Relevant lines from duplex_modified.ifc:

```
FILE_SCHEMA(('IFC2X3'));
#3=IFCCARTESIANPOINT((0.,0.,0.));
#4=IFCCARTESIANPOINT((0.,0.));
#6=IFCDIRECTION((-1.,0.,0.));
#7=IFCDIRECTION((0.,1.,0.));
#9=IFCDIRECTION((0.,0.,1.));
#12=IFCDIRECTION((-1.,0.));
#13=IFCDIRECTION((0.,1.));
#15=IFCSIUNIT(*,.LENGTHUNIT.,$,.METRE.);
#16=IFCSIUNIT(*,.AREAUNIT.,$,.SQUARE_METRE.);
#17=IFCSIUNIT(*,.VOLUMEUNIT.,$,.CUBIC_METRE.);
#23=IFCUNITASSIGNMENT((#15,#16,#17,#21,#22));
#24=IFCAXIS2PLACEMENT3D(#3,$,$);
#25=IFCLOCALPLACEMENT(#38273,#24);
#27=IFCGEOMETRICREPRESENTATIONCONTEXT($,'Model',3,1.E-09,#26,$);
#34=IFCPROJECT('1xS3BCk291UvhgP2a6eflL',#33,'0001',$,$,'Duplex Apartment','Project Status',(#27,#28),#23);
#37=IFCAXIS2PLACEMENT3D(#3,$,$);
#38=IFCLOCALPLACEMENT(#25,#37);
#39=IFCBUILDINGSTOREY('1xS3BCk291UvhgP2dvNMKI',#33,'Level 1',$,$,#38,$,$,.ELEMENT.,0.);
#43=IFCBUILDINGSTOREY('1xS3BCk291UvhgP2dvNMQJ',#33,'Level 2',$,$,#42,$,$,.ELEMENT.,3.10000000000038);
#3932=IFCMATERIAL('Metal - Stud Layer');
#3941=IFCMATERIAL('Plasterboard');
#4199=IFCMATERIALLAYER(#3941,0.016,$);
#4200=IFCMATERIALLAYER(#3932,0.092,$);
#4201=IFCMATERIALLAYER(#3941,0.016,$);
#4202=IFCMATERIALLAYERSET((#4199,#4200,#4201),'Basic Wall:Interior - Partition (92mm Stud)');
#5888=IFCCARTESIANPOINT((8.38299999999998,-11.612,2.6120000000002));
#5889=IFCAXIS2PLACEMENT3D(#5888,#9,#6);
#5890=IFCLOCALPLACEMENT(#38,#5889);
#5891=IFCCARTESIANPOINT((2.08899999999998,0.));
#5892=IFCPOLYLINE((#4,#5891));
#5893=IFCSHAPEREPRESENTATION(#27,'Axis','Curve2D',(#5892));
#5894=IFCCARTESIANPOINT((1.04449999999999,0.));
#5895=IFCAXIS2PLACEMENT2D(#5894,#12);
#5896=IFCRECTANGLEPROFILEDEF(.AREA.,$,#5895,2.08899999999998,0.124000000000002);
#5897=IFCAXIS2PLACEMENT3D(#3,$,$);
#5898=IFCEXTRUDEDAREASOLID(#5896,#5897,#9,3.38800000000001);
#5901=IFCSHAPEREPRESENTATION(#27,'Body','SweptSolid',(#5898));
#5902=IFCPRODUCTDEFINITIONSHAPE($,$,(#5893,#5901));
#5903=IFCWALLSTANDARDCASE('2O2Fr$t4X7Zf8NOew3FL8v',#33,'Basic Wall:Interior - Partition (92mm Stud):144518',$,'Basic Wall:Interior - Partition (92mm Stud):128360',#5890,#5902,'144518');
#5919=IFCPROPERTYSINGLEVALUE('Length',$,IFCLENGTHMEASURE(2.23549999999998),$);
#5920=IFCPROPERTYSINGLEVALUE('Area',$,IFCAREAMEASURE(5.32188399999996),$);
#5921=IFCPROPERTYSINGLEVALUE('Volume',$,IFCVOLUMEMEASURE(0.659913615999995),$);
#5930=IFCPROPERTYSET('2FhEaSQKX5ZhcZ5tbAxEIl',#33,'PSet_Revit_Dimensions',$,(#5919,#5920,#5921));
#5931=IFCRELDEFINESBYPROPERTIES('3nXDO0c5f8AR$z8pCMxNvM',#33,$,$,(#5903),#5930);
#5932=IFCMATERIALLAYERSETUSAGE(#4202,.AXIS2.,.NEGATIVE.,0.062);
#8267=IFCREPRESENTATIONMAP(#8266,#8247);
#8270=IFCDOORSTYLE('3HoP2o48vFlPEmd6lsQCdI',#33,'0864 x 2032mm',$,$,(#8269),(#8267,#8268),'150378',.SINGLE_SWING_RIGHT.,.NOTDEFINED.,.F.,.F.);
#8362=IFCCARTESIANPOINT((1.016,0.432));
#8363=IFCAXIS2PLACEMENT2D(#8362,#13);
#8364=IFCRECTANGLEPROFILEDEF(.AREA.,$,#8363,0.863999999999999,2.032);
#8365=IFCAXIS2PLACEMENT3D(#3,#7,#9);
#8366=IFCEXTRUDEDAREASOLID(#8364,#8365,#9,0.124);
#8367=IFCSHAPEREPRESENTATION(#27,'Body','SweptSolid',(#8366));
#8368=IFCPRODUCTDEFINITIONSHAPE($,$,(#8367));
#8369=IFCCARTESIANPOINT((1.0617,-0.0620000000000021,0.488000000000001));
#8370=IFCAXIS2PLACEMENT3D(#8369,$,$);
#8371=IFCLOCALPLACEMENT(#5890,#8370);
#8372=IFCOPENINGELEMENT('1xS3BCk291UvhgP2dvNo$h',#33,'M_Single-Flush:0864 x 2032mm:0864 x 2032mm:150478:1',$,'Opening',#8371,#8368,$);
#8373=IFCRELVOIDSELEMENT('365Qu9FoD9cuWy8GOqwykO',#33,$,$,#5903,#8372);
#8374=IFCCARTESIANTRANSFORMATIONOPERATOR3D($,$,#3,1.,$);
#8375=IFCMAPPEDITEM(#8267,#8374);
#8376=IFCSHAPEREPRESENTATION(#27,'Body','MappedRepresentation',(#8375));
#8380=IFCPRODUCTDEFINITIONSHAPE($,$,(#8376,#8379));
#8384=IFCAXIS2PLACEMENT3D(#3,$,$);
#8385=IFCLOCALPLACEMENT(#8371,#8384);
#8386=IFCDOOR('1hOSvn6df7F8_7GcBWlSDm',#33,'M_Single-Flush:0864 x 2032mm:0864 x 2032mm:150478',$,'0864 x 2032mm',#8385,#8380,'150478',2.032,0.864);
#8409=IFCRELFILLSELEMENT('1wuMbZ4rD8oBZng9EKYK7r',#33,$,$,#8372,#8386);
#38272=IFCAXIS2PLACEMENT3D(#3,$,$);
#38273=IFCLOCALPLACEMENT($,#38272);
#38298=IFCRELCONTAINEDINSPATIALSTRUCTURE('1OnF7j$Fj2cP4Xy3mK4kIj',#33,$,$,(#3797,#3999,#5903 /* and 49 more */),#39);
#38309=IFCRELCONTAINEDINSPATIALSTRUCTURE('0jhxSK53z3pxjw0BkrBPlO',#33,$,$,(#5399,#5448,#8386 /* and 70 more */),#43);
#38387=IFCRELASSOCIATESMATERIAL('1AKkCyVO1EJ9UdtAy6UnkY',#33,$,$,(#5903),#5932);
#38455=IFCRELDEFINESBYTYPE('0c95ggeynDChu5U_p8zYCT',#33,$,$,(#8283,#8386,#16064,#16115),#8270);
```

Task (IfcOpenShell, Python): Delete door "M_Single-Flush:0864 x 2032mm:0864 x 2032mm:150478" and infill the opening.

```python
import ifcopenshell
import ifcopenshell.api.feature
import ifcopenshell.api.pset
import ifcopenshell.api.root
import ifcopenshell.geom
import ifcopenshell.util.element
import ifcopenshell.util.shape
import ifcopenshell.util.unit

model = ifcopenshell.open("duplex_modified.ifc")
area_scale = ifcopenshell.util.unit.calculate_unit_scale(model, "AREAUNIT")
volume_scale = ifcopenshell.util.unit.calculate_unit_scale(model, "VOLUMEUNIT")
settings = ifcopenshell.geom.settings()


def volume(element):
    """Net volume in cubic metres, openings subtracted."""
    shape = ifcopenshell.geom.create_shape(settings, element)
    return ifcopenshell.util.shape.get_volume(shape.geometry)


door = model.by_guid("1hOSvn6df7F8_7GcBWlSDm")
opening = door.FillsVoids[0].RelatingOpeningElement
wall = opening.VoidsElements[0].RelatingBuildingElement
before = volume(wall)

ifcopenshell.api.root.remove_product(model, product=door)
ifcopenshell.api.feature.remove_feature(model, feature=opening)

after = volume(wall)
thickness = 0.124  # wall thickness in metres

# Update the wall's stored quantities.
pset = model.by_id(ifcopenshell.util.element.get_pset(wall, "PSet_Revit_Dimensions", should_inherit=False)["id"])
ifcopenshell.api.pset.edit_pset(model, pset=pset, properties={
    "Area": model.create_entity("IfcAreaMeasure", after / thickness / area_scale),
    "Volume": model.create_entity("IfcVolumeMeasure", after / volume_scale),
})

print(f"wall volume {before:.3f} -> {after:.3f} m3")

model.write("duplex_modified_updated.ifc")
```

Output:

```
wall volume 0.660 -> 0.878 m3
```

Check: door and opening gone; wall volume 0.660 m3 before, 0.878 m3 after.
